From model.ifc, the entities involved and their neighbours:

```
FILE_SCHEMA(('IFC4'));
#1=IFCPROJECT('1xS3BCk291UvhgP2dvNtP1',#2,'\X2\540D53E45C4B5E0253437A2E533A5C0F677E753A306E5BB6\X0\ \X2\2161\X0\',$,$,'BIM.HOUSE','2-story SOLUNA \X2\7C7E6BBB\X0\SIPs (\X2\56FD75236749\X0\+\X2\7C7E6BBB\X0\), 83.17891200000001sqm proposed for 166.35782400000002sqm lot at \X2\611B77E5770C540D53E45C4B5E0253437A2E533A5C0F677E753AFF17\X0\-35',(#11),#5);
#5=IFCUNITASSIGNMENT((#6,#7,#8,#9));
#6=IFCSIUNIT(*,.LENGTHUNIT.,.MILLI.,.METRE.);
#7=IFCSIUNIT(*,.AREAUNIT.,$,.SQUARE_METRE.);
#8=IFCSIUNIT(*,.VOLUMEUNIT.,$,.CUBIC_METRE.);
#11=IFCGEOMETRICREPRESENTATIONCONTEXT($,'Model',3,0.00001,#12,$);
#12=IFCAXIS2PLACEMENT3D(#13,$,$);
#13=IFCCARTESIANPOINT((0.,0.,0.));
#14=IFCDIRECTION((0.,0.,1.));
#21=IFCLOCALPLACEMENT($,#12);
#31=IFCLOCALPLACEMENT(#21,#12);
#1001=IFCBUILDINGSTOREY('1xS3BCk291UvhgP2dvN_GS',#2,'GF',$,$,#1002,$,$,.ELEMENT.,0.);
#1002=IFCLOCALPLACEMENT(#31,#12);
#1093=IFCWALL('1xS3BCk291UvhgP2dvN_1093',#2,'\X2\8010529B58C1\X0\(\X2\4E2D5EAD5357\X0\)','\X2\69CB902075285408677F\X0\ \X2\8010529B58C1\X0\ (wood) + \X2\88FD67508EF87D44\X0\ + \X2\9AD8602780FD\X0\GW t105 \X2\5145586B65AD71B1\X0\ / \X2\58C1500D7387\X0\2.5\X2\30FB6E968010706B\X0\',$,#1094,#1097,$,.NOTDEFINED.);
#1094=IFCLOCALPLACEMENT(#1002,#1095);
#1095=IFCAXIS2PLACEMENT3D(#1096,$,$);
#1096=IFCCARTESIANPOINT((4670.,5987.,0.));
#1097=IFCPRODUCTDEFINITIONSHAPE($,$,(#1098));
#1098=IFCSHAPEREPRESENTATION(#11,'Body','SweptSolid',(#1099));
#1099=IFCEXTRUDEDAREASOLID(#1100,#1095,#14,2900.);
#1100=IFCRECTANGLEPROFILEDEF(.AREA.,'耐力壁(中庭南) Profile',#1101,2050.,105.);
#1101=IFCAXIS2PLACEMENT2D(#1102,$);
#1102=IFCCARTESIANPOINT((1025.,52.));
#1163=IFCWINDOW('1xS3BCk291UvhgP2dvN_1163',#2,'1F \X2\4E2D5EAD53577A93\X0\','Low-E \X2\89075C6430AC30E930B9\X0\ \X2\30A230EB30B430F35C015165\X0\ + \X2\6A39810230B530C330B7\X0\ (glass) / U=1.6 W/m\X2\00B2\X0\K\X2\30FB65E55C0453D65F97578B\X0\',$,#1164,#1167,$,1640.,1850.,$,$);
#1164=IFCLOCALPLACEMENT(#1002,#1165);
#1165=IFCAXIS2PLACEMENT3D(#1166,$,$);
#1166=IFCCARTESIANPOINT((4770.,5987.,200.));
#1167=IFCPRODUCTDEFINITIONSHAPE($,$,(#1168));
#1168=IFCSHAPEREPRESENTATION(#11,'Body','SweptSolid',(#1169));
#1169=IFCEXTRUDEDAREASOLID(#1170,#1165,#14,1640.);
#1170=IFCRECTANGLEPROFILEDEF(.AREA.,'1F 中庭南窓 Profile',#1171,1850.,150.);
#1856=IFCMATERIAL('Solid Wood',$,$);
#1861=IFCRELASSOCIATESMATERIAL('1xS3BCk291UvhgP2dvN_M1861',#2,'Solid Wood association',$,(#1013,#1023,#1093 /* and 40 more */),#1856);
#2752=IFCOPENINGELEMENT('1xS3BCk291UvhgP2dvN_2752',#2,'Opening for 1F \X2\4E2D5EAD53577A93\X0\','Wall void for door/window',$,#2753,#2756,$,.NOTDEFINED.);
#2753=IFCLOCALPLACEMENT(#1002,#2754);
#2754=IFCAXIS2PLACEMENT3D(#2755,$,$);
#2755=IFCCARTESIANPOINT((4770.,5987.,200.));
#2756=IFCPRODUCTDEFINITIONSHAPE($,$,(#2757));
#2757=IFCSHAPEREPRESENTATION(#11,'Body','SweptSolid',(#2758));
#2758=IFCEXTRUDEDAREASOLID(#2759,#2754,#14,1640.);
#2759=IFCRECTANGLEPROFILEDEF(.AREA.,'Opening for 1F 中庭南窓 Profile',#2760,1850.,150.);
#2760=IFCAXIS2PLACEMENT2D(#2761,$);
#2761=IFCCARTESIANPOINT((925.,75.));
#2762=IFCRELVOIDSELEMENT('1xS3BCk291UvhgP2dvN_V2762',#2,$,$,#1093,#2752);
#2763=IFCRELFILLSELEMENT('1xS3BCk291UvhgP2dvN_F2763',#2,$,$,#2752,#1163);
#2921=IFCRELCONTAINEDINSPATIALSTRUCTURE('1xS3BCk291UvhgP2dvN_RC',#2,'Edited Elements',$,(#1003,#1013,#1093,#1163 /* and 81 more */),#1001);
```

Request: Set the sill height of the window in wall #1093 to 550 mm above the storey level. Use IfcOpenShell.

```python
import numpy as np
import ifcopenshell
import ifcopenshell.api.geometry
import ifcopenshell.geom
import ifcopenshell.util.element
import ifcopenshell.util.placement
import ifcopenshell.util.shape
import ifcopenshell.util.unit

model = ifcopenshell.open("model.ifc")
unit_scale = ifcopenshell.util.unit.calculate_unit_scale(model)

window = model.by_id(1163)
opening = window.FillsVoids[0].RelatingOpeningElement
storey = ifcopenshell.util.element.get_container(window, ifc_class="IfcBuildingStorey")
level = ifcopenshell.util.placement.get_local_placement(storey.ObjectPlacement)[2, 3]

# The opening's origin need not be at the sill, so measure its lowest point.
shape = ifcopenshell.geom.create_shape(ifcopenshell.geom.settings(), opening)
bottom = ifcopenshell.util.shape.get_shape_bottom_elevation(shape, shape.geometry) / unit_scale
dz = level + 0.55 / unit_scale - bottom

shift = np.array([0.0, 0.0, dz])
# The window is not placed relative to its opening, so move both.
for product in (opening, window):
    matrix = ifcopenshell.util.placement.get_local_placement(product.ObjectPlacement)
    matrix[:3, 3] += shift
    ifcopenshell.api.geometry.edit_object_placement(model, product=product, matrix=matrix, is_si=False)

print(f"moved by {dz * unit_scale:+.3f} m")

model.write("model_updated.ifc")
```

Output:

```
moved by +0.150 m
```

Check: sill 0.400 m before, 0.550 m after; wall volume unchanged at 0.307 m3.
